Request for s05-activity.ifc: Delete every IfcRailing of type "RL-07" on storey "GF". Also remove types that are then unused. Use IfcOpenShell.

First a look at what the model holds.

```python
import ifcopenshell
import ifcopenshell.util.element

model = ifcopenshell.open("s05-activity.ifc")
print(model.schema)
storey = next(s for s in model.by_type("IfcBuildingStorey") if s.Name == "GF")
railings = [e for e in ifcopenshell.util.element.get_decomposition(storey) if e.is_a("IfcRailing")]
seen = {}
for e in railings:
    element_type = ifcopenshell.util.element.get_type(e)
    name = element_type.Name if element_type not in (None, e) else None
    seen[name] = seen.get(name, 0) + 1
for name, count in sorted(seen.items(), key=str):
    print(count, "x", name)
```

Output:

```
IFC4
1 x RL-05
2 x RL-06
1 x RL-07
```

```python
import ifcopenshell
import ifcopenshell.api.root
import ifcopenshell.util.element

model = ifcopenshell.open("s05-activity.ifc")

storey = next(s for s in model.by_type("IfcBuildingStorey") if s.Name == "GF")
railings = [e for e in ifcopenshell.util.element.get_decomposition(storey) if e.is_a("IfcRailing")]
targets = [e for e in railings if (t := ifcopenshell.util.element.get_type(e)) not in (None, e) and t.Name == "RL-07"]
types = {ifcopenshell.util.element.get_type(e) for e in targets} - {None, *targets}

for e in targets:
    ifcopenshell.api.root.remove_product(model, product=e)
print(len(targets), "removed")

unused = [t for t in types if not ifcopenshell.util.element.get_types(t)]
for t in unused:
    ifcopenshell.api.root.remove_product(model, product=t)
print(len(unused), "unused types removed")

model.write("s05-activity_rev.ifc")
```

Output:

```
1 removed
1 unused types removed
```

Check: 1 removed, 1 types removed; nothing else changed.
